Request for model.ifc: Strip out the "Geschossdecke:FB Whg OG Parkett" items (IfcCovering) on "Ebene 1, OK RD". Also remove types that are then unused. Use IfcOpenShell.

First a look at what the model holds.

```python
import ifcopenshell
import ifcopenshell.util.element

model = ifcopenshell.open("model.ifc")
print(model.schema)
storey = next(s for s in model.by_type("IfcBuildingStorey") if s.Name == "Ebene 1, OK RD")
coverings = [e for e in ifcopenshell.util.element.get_decomposition(storey) if e.is_a("IfcCovering")]
seen = {}
for e in coverings:
    element_type = ifcopenshell.util.element.get_type(e)
    name = element_type.Name if element_type not in (None, e) else None
    seen[name] = seen.get(name, 0) + 1
for name, count in sorted(seen.items(), key=str):
    print(count, "x", name)
```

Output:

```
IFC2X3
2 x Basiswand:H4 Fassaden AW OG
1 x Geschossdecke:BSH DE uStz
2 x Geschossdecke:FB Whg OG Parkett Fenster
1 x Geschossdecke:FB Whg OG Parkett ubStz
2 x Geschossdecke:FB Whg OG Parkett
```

```python
import ifcopenshell
import ifcopenshell.api.root
import ifcopenshell.util.element

model = ifcopenshell.open("model.ifc")

storey = next(s for s in model.by_type("IfcBuildingStorey") if s.Name == "Ebene 1, OK RD")
coverings = [e for e in ifcopenshell.util.element.get_decomposition(storey) if e.is_a("IfcCovering")]
targets = [e for e in coverings if (t := ifcopenshell.util.element.get_type(e)) not in (None, e) and t.Name == "Geschossdecke:FB Whg OG Parkett"]
types = {ifcopenshell.util.element.get_type(e) for e in targets} - {None, *targets}

for e in targets:
    ifcopenshell.api.root.remove_product(model, product=e)
print(len(targets), "removed")

unused = [t for t in types if not ifcopenshell.util.element.get_types(t)]
for t in unused:
    ifcopenshell.api.root.remove_product(model, product=t)
print(len(unused), "unused types removed")

model.write("model_rev.ifc")
```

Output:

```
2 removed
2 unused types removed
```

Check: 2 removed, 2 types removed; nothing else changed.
